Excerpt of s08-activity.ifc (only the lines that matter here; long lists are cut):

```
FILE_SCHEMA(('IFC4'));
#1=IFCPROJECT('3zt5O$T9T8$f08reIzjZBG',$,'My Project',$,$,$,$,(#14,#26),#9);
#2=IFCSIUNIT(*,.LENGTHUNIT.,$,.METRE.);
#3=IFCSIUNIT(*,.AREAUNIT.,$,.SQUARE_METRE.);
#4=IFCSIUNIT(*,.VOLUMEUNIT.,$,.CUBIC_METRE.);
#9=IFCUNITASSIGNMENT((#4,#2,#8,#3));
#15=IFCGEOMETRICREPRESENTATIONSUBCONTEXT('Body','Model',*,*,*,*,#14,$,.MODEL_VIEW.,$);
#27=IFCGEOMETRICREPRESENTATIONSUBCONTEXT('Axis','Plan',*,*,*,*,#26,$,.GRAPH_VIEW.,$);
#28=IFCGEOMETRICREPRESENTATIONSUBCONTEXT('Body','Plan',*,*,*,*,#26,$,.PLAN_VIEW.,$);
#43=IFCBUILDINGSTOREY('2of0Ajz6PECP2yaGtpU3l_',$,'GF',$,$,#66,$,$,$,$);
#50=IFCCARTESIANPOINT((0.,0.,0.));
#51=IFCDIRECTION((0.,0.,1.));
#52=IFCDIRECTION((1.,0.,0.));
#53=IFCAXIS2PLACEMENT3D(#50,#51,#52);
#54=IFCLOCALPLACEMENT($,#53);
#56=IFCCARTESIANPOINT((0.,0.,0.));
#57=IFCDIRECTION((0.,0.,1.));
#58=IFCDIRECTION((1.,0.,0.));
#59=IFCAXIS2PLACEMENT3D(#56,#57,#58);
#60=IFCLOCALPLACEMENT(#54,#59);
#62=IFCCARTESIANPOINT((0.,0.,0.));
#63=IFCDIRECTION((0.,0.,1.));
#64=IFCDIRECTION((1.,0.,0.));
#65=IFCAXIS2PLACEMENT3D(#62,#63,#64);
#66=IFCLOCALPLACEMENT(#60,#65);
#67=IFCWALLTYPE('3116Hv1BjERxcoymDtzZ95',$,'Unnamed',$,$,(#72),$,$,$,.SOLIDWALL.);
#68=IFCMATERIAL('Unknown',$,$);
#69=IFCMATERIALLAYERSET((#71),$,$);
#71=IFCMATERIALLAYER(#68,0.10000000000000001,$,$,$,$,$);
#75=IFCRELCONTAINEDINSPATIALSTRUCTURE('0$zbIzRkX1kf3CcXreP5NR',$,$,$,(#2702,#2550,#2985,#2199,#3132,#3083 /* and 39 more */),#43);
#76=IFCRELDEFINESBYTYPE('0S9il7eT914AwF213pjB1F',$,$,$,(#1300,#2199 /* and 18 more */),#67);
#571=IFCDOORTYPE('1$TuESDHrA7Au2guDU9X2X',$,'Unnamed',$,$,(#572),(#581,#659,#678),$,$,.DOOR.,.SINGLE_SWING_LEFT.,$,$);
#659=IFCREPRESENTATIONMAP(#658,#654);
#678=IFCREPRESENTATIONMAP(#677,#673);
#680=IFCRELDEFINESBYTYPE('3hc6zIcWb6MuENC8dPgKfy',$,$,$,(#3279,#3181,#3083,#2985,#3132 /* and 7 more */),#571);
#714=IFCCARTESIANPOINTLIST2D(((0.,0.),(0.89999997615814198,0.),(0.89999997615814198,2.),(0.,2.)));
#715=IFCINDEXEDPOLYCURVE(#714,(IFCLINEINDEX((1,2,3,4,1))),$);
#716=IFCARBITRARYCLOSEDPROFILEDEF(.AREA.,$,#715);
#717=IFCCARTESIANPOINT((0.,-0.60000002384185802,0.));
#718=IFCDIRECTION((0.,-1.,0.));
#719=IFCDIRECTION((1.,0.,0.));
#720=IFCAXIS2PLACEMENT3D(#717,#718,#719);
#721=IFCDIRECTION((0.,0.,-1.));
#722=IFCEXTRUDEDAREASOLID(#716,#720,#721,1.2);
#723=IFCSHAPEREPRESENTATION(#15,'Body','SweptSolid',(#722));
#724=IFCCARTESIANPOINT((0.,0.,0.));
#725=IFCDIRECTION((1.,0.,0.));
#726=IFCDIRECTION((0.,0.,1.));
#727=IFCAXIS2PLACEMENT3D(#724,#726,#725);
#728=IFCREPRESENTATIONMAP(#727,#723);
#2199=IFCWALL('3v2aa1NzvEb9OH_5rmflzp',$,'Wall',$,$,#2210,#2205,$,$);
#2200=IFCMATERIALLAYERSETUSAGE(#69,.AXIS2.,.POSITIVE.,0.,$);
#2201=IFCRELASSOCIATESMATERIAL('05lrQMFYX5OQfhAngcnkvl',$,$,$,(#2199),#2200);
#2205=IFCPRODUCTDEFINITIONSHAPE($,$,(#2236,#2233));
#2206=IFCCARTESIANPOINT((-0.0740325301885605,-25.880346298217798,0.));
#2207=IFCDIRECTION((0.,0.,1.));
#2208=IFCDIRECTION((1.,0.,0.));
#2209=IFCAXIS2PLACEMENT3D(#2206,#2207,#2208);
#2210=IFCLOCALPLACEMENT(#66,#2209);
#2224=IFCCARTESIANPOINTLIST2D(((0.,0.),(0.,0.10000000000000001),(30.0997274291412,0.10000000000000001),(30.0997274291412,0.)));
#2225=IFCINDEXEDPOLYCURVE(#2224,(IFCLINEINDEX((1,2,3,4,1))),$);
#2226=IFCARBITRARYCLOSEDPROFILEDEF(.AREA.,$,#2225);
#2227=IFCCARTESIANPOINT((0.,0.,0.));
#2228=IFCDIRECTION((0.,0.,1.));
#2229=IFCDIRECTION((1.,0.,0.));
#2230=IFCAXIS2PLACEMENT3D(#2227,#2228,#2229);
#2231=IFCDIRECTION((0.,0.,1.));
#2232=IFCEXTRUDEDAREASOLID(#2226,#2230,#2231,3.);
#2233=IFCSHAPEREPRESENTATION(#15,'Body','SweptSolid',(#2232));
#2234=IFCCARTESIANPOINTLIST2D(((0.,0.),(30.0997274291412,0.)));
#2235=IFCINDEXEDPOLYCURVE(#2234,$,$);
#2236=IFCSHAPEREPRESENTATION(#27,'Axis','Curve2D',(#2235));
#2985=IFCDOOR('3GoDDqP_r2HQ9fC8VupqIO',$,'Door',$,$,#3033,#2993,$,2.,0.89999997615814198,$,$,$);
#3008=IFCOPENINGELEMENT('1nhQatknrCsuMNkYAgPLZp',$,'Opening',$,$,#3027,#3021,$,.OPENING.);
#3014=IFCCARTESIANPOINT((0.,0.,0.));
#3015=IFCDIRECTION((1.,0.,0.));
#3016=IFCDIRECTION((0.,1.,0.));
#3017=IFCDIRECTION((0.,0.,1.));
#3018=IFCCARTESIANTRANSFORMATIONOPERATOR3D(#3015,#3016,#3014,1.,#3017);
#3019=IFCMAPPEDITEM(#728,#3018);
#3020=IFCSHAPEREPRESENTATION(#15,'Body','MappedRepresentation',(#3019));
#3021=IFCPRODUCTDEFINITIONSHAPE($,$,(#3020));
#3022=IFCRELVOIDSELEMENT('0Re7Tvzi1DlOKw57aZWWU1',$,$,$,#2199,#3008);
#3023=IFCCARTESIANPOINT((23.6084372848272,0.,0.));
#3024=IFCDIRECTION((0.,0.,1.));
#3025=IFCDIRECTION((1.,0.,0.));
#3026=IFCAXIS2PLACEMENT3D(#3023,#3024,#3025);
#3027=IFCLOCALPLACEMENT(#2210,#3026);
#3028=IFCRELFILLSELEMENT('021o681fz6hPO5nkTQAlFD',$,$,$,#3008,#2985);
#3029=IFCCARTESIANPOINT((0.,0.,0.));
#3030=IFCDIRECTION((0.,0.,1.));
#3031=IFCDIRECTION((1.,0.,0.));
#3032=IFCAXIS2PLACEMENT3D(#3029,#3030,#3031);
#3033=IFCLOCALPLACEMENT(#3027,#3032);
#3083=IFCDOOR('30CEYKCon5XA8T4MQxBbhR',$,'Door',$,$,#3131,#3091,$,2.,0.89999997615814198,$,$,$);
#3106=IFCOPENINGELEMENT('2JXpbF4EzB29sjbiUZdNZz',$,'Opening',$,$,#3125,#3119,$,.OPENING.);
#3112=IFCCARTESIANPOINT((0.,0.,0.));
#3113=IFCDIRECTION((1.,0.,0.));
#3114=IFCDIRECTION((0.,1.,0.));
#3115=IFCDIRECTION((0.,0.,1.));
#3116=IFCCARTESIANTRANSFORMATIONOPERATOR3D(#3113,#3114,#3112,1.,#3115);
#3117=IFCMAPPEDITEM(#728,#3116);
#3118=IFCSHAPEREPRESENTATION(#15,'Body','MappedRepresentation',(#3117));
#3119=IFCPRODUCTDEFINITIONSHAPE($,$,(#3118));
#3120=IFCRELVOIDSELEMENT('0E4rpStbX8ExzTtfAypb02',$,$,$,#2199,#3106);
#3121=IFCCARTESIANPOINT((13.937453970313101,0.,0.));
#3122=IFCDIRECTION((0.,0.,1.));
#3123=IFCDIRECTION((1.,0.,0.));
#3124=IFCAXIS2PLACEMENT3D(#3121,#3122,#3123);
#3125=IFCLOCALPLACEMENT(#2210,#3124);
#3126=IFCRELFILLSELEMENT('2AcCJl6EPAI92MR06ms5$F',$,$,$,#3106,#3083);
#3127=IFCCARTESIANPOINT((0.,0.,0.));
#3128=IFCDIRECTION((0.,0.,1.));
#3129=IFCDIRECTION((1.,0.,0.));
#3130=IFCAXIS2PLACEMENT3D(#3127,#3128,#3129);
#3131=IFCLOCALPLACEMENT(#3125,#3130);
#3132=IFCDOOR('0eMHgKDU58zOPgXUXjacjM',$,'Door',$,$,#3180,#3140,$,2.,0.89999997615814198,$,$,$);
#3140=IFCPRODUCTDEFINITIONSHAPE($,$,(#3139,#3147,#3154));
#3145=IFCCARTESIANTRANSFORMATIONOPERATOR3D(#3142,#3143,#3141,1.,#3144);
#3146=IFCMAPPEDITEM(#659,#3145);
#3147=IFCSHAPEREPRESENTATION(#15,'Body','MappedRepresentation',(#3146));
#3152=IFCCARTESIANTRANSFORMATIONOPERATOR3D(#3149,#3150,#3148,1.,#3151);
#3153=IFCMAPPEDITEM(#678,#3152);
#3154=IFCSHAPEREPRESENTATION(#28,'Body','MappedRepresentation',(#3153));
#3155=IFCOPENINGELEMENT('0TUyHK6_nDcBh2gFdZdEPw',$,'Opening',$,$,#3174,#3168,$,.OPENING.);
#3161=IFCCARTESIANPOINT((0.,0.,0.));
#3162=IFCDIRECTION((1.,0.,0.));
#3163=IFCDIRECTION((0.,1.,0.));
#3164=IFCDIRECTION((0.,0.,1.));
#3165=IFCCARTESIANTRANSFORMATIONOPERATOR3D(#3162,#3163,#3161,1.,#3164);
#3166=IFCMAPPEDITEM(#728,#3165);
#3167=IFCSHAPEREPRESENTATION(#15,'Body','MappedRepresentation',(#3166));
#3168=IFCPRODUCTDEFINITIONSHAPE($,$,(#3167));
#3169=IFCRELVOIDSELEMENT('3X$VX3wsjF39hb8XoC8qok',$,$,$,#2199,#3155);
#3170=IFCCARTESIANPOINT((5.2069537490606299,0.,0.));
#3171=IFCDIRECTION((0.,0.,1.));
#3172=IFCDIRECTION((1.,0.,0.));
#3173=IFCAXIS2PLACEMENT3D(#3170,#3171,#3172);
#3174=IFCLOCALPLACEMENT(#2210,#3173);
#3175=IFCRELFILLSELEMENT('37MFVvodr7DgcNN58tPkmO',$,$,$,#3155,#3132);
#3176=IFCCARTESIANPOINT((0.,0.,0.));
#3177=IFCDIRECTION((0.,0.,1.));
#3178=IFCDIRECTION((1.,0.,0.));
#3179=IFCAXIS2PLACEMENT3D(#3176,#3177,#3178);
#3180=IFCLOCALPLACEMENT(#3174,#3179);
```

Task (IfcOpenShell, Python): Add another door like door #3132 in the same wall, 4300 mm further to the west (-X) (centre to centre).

```python
import ifcopenshell
import ifcopenshell.api.feature
import ifcopenshell.api.geometry
import ifcopenshell.api.root
import ifcopenshell.geom
import ifcopenshell.util.element
import ifcopenshell.util.placement
import ifcopenshell.util.shape
import ifcopenshell.util.unit

model = ifcopenshell.open("s08-activity.ifc")
unit_scale = ifcopenshell.util.unit.calculate_unit_scale(model)
settings = ifcopenshell.geom.settings()


def volume(element):
    """Net volume in cubic metres, openings subtracted."""
    shape = ifcopenshell.geom.create_shape(settings, element)
    return ifcopenshell.util.shape.get_volume(shape.geometry)


door = model.by_guid("0eMHgKDU58zOPgXUXjacjM")
opening = door.FillsVoids[0].RelatingOpeningElement
wall = opening.VoidsElements[0].RelatingBuildingElement
before = volume(wall)
shift = ifcopenshell.util.placement.get_local_placement(wall.ObjectPlacement)[:3, 0] * -4.3 / unit_scale

# copy_class copies the void relationship, type, container and properties, but no geometry.
new_opening = ifcopenshell.api.root.copy_class(model, product=opening)
new_opening.Representation = ifcopenshell.util.element.copy_deep(
    model, opening.Representation, exclude=["IfcGeometricRepresentationContext", "IfcRepresentationMap"]
)
new_door = ifcopenshell.api.root.copy_class(model, product=door)
new_door.Representation = ifcopenshell.util.element.copy_deep(
    model, door.Representation, exclude=["IfcGeometricRepresentationContext", "IfcRepresentationMap"]
)
ifcopenshell.api.feature.add_filling(model, opening=new_opening, element=new_door)

for old, new in ((opening, new_opening), (door, new_door)):
    matrix = ifcopenshell.util.placement.get_local_placement(old.ObjectPlacement)
    matrix[:3, 3] += shift
    ifcopenshell.api.geometry.edit_object_placement(model, product=new, matrix=matrix, is_si=False)

after = volume(wall)

print(f"wall volume {before:.3f} -> {after:.3f} m3")

model.write("s08-activity-out.ifc")
```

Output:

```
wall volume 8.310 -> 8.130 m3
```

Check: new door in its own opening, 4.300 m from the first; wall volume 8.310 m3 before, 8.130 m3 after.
